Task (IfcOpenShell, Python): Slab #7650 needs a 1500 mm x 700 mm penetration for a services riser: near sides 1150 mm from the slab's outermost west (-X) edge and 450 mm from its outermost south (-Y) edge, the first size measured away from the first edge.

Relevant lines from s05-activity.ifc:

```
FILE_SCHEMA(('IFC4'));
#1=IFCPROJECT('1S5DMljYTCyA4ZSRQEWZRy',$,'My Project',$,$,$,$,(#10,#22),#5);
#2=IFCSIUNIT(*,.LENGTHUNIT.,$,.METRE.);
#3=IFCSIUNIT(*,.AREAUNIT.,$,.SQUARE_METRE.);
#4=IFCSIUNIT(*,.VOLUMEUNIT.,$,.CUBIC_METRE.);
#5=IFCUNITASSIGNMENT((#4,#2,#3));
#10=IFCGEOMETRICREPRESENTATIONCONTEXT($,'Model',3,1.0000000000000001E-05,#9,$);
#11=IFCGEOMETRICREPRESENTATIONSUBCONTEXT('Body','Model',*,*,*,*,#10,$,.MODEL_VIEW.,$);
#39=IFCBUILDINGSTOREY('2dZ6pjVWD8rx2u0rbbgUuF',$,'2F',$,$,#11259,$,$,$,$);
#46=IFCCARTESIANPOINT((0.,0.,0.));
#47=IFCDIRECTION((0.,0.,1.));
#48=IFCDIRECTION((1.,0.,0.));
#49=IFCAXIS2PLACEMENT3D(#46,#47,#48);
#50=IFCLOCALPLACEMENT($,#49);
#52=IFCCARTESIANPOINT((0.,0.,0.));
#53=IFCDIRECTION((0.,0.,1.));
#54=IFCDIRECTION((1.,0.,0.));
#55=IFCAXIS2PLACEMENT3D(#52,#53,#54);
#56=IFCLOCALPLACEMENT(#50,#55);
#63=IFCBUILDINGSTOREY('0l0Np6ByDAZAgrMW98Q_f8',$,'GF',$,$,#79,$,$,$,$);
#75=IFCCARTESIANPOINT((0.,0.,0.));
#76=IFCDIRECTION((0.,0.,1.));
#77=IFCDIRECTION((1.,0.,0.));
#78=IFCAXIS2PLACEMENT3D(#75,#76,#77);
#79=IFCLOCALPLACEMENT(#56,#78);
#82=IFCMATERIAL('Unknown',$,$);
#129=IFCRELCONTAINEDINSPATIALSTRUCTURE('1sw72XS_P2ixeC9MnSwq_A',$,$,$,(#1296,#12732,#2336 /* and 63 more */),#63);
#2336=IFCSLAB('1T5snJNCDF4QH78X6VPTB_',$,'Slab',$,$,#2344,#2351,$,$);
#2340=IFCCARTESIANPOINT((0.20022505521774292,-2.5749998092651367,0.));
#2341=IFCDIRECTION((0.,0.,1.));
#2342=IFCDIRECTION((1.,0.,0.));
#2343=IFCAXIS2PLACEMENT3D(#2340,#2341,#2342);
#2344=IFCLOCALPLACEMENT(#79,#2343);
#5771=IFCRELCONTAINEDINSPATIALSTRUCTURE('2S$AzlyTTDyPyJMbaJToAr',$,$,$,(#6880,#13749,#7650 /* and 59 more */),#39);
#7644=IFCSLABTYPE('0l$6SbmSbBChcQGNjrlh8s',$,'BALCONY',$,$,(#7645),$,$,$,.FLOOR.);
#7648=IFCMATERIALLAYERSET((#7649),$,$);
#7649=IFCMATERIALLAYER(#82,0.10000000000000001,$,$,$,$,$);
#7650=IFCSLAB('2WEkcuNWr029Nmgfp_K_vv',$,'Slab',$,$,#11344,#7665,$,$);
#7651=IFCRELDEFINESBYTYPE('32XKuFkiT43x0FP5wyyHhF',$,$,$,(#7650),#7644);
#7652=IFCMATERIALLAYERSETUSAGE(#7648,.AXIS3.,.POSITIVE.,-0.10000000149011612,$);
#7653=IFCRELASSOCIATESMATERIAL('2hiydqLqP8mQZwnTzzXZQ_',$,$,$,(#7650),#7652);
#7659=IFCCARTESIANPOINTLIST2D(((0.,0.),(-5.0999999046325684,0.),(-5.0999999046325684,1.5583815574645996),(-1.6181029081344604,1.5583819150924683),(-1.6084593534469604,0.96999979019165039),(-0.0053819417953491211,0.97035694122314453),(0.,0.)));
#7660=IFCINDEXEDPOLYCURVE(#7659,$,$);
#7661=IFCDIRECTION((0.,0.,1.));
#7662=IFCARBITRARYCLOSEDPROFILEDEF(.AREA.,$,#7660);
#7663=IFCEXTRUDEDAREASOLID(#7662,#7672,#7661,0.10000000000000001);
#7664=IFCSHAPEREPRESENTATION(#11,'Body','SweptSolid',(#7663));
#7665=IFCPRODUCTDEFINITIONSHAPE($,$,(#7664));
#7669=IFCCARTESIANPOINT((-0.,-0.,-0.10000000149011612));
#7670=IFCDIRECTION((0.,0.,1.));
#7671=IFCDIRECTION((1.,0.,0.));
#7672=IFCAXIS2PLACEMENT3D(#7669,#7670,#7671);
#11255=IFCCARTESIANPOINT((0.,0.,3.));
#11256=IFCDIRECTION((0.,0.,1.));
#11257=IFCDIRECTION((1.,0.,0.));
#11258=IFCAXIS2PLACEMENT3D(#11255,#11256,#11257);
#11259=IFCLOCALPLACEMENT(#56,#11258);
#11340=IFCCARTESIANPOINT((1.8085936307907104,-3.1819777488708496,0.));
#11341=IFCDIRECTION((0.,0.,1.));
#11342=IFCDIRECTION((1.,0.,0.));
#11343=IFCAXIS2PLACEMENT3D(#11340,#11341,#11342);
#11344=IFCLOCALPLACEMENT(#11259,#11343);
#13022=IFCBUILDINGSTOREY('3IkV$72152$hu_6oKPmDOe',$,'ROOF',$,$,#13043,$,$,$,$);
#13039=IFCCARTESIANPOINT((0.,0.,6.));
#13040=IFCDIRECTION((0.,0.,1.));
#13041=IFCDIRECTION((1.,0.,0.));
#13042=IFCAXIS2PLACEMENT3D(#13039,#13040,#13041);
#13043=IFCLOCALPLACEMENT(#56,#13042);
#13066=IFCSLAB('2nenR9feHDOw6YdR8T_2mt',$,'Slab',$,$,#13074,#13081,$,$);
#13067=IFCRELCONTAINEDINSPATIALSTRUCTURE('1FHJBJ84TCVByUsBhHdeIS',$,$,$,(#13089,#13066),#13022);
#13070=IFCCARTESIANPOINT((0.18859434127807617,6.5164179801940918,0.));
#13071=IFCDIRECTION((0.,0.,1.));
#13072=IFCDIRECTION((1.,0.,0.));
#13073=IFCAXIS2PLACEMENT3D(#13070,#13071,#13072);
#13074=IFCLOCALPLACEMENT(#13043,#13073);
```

```python
import numpy as np
import ifcopenshell
import ifcopenshell.api.feature
import ifcopenshell.api.geometry
import ifcopenshell.api.root
import ifcopenshell.geom
import ifcopenshell.util.placement
import ifcopenshell.util.representation
import ifcopenshell.util.shape
import ifcopenshell.util.unit

model = ifcopenshell.open("s05-activity.ifc")
unit_scale = ifcopenshell.util.unit.calculate_unit_scale(model)
settings = ifcopenshell.geom.settings()


def volume(element):
    """Net volume in cubic metres, openings subtracted."""
    shape = ifcopenshell.geom.create_shape(settings, element)
    return ifcopenshell.util.shape.get_volume(shape.geometry)


slab = model.by_guid("2WEkcuNWr029Nmgfp_K_vv")
before = volume(slab)

# Extent in the slab's own axes, in metres. The edges named are its -X and -Y sides.
slab_shape = ifcopenshell.geom.create_shape(settings, slab)
vertices = ifcopenshell.util.shape.get_vertices(slab_shape.geometry)
x_min, y_min, bottom = vertices.min(axis=0)
top = vertices[:, 2].max()

opening = ifcopenshell.api.root.create_entity(model, ifc_class="IfcOpeningElement", name="Services riser opening", predefined_type="OPENING")
context = ifcopenshell.util.representation.get_context(model, "Model", "Body", "MODEL_VIEW")
width, depth = 1.5, 0.7
outline = [(0.0, 0.0), (width, 0.0), (width, depth), (0.0, depth), (0.0, 0.0)]
# Overshoot both faces by 50 mm so the cut is clean.
shape = ifcopenshell.api.geometry.add_slab_representation(
    model, context=context, depth=top - bottom + 0.1, polyline=outline
)
ifcopenshell.api.geometry.assign_representation(model, product=opening, representation=shape)

matrix = ifcopenshell.util.placement.get_local_placement(slab.ObjectPlacement)
matrix[:, 3] = matrix @ np.append(np.array([x_min + 1.15, y_min + 0.45, bottom - 0.05]) / unit_scale, 1.0)
ifcopenshell.api.geometry.edit_object_placement(model, product=opening, matrix=matrix, is_si=False)
ifcopenshell.api.feature.add_feature(model, feature=opening, element=slab)

after = volume(slab)

print(f"slab volume {before:.3f} -> {after:.3f} m3")

model.write("s05-activity_v2.ifc")
```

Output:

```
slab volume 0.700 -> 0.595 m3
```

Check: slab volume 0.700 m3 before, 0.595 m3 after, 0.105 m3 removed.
